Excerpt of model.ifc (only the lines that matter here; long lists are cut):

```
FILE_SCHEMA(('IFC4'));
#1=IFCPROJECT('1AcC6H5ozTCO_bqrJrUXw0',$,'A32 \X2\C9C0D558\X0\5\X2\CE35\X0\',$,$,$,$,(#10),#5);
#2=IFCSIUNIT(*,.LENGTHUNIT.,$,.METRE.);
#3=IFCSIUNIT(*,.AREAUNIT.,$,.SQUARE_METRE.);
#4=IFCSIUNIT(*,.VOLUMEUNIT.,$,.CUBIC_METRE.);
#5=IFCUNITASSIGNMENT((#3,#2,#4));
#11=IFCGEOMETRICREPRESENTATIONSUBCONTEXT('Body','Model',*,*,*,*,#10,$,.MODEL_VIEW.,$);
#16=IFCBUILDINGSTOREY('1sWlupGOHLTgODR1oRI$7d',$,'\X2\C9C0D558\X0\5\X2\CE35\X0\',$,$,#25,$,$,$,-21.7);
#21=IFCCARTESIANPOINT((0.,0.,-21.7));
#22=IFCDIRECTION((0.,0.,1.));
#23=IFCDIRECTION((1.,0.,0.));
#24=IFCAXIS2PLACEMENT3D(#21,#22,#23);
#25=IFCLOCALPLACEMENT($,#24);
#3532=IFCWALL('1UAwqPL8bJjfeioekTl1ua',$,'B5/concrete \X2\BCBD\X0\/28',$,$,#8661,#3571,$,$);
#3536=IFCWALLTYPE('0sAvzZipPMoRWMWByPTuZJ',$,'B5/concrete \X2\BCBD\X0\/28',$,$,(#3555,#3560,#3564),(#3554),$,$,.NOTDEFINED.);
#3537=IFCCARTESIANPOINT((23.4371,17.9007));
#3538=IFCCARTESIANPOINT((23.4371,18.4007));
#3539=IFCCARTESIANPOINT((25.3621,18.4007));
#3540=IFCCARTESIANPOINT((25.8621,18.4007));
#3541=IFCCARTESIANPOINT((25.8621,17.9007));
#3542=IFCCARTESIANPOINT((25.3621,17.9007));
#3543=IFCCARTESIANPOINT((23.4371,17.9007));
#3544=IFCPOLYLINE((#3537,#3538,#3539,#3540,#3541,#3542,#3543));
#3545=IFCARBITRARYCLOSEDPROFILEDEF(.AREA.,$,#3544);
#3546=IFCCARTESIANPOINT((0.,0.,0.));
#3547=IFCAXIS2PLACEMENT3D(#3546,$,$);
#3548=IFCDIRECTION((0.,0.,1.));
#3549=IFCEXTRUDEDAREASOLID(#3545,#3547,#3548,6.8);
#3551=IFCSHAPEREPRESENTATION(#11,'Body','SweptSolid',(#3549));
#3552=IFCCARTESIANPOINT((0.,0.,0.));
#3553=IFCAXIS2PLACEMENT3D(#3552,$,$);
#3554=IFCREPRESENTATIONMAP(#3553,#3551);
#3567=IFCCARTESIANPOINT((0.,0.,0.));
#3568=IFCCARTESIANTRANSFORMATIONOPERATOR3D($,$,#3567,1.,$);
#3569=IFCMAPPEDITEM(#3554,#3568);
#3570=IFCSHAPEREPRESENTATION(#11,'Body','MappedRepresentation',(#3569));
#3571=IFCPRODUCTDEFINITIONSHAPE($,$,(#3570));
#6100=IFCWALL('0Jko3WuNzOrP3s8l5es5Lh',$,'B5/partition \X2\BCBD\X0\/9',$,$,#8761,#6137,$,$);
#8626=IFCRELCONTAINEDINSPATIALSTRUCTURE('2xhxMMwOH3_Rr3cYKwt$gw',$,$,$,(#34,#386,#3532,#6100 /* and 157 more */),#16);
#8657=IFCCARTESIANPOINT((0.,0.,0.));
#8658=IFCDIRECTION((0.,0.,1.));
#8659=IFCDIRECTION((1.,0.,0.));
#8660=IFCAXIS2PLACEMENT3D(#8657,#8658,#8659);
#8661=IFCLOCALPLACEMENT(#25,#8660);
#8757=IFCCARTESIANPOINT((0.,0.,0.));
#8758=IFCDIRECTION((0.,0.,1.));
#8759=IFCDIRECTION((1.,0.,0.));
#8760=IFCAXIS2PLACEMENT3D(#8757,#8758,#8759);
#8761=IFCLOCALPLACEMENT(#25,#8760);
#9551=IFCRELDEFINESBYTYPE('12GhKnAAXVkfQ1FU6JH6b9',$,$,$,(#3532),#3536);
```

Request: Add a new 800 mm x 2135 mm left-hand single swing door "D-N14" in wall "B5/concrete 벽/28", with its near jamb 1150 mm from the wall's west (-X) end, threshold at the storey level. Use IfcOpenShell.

```python
import numpy as np
import ifcopenshell
import ifcopenshell.api.feature
import ifcopenshell.api.geometry
import ifcopenshell.api.root
import ifcopenshell.api.spatial
import ifcopenshell.geom
import ifcopenshell.util.element
import ifcopenshell.util.placement
import ifcopenshell.util.representation
import ifcopenshell.util.shape
import ifcopenshell.util.unit

model = ifcopenshell.open("model.ifc")
unit_scale = ifcopenshell.util.unit.calculate_unit_scale(model)
settings = ifcopenshell.geom.settings()


def volume(element):
    """Net volume in cubic metres, openings subtracted."""
    shape = ifcopenshell.geom.create_shape(settings, element)
    return ifcopenshell.util.shape.get_volume(shape.geometry)


wall = model.by_guid("1UAwqPL8bJjfeioekTl1ua")
storey = ifcopenshell.util.element.get_container(wall, ifc_class="IfcBuildingStorey")
context = ifcopenshell.util.representation.get_context(model, "Model", "Body", "MODEL_VIEW")
before = volume(wall)

width, height, from_end, sill = 0.8, 2.135, 1.15, 0.0  # metres

# The wall runs along its own X axis, and the end named is its -X end.
wall_shape = ifcopenshell.geom.create_shape(settings, wall)
x, y, z = ifcopenshell.util.shape.get_vertices(wall_shape.geometry).T
start = x.min() + from_end
face, thickness = float(y.min()), float(y.max() - y.min())
wall_matrix = ifcopenshell.util.placement.get_local_placement(wall.ObjectPlacement)
level = ifcopenshell.util.placement.get_local_placement(storey.ObjectPlacement)[2, 3]


def in_wall(x, y):
    """Placement at x, y metres in the wall's axes, at sill height."""
    matrix = wall_matrix.copy()
    matrix[:, 3] = wall_matrix @ np.array([x / unit_scale, y / unit_scale, 0.0, 1.0])
    matrix[2, 3] = level + sill / unit_scale
    return matrix


# Opening: a box that overshoots both wall faces by 50 mm.
opening = ifcopenshell.api.root.create_entity(model, ifc_class="IfcOpeningElement", predefined_type="OPENING")
box = ifcopenshell.api.geometry.add_wall_representation(
    model, context=context, length=width, height=height, thickness=thickness + 0.1
)
ifcopenshell.api.geometry.assign_representation(model, product=opening, representation=box)
ifcopenshell.api.geometry.edit_object_placement(model, product=opening, matrix=in_wall(start, face - 0.05), is_si=False)
ifcopenshell.api.feature.add_feature(model, feature=opening, element=wall)

door = ifcopenshell.api.root.create_entity(model, ifc_class="IfcDoor", name="D-N14", predefined_type="DOOR")
door.OverallWidth, door.OverallHeight = width / unit_scale, height / unit_scale
door.OperationType = "SINGLE_SWING_LEFT"
body = ifcopenshell.api.geometry.add_door_representation(
    model,
    context=context,
    overall_width=door.OverallWidth,
    overall_height=door.OverallHeight,
    operation_type="SINGLE_SWING_LEFT",
    lining_properties={"LiningDepth": thickness / unit_scale, "ThresholdDepth": thickness / unit_scale},
)
ifcopenshell.api.geometry.assign_representation(model, product=door, representation=body)
ifcopenshell.api.spatial.assign_container(model, products=[door], relating_structure=storey)
ifcopenshell.api.feature.add_filling(model, opening=opening, element=door)

# The lining spans the wall, so the door starts at the wall face.
ifcopenshell.api.geometry.edit_object_placement(model, product=door, matrix=in_wall(start, face), is_si=False)

after = volume(wall)

print(f"wall volume {before:.3f} -> {after:.3f} m3")

model.write("model_v2.ifc")
```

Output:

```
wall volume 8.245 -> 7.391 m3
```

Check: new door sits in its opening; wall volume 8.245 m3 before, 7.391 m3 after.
